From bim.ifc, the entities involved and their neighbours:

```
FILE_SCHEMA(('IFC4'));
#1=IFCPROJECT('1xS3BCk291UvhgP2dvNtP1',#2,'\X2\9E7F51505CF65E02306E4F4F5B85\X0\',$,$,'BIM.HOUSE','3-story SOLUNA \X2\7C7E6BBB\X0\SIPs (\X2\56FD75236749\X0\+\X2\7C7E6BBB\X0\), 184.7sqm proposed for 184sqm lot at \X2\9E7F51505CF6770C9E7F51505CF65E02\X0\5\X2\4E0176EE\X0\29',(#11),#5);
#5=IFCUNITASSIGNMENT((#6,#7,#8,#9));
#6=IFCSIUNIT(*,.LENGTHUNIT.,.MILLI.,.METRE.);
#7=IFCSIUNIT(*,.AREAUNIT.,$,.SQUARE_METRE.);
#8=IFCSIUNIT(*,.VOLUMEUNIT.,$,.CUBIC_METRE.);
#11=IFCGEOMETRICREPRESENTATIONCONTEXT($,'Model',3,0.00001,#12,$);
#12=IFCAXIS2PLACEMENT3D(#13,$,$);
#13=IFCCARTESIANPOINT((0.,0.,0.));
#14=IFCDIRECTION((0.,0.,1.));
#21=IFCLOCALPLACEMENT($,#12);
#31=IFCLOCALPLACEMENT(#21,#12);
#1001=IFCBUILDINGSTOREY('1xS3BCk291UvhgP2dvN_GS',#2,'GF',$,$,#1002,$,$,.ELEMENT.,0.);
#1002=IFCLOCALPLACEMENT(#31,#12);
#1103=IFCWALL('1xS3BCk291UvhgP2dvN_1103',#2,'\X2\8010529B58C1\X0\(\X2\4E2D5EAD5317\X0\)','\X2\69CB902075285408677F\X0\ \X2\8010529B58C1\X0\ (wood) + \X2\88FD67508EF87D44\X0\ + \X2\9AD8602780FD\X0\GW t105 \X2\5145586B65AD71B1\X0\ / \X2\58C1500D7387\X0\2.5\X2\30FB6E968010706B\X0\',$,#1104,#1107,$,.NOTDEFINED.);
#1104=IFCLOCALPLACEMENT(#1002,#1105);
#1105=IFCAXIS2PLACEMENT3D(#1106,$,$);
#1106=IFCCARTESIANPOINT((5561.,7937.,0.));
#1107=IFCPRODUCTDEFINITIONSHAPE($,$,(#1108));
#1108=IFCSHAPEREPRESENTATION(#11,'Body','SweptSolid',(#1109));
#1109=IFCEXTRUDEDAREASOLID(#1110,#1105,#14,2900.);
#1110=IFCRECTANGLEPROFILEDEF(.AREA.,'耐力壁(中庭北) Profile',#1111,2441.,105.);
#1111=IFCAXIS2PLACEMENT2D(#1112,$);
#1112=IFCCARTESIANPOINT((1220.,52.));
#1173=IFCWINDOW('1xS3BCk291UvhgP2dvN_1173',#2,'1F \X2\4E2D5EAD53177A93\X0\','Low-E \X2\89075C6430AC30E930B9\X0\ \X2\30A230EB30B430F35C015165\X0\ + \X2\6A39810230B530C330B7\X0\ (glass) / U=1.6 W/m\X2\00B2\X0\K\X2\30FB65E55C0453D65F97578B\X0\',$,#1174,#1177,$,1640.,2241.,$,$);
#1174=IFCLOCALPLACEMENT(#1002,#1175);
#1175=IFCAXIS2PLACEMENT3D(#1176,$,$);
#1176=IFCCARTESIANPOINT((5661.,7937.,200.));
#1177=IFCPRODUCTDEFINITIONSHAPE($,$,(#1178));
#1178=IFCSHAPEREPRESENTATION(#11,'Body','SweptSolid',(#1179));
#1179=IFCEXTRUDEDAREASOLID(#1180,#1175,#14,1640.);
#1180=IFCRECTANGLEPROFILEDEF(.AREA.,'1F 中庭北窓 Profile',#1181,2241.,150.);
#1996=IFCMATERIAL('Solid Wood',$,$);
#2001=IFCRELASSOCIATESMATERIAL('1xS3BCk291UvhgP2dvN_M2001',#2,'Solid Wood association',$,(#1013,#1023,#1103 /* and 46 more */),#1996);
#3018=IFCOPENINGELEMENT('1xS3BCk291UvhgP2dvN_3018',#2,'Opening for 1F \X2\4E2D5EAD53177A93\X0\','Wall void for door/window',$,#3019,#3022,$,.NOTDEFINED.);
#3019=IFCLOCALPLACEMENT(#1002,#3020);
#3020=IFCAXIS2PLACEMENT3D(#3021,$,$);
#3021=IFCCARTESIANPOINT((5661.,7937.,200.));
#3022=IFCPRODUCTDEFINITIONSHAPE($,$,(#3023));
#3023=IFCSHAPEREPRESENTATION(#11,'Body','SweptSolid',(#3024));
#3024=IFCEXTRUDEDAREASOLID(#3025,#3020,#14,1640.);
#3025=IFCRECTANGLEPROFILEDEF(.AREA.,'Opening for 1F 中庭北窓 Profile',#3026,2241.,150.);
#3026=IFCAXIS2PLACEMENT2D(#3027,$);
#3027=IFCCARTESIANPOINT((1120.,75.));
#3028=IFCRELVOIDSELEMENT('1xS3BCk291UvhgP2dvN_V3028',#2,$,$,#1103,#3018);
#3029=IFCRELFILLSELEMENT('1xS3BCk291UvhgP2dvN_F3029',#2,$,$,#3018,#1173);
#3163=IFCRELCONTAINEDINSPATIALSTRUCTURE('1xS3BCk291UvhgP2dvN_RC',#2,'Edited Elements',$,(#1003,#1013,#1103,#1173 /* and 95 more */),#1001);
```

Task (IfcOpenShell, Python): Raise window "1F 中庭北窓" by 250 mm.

```python
import numpy as np
import ifcopenshell
import ifcopenshell.api.geometry
import ifcopenshell.util.placement
import ifcopenshell.util.unit

model = ifcopenshell.open("bim.ifc")
unit_scale = ifcopenshell.util.unit.calculate_unit_scale(model)

window = model.by_guid("1xS3BCk291UvhgP2dvN_1173")
opening = window.FillsVoids[0].RelatingOpeningElement
dz = 0.25 / unit_scale

shift = np.array([0.0, 0.0, dz])
# The window is not placed relative to its opening, so move both.
for product in (opening, window):
    matrix = ifcopenshell.util.placement.get_local_placement(product.ObjectPlacement)
    matrix[:3, 3] += shift
    ifcopenshell.api.geometry.edit_object_placement(model, product=product, matrix=matrix, is_si=False)

print(f"moved by {dz * unit_scale:+.3f} m")

model.write("bim_v2.ifc")
```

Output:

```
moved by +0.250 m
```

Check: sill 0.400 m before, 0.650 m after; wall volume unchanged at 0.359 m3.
